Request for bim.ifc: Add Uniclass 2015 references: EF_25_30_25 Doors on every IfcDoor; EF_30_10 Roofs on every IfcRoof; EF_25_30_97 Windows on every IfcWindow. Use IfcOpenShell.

First a look at what the model holds.

```python
import ifcopenshell

model = ifcopenshell.open("bim.ifc")
print(model.schema)
print("classifications:", [c.Name for c in model.by_type("IfcClassification")])
for ifc_class in ("IfcDoor", "IfcRoof", "IfcStair", "IfcWall", "IfcWindow"):
    print(ifc_class, len(model.by_type(ifc_class)))
```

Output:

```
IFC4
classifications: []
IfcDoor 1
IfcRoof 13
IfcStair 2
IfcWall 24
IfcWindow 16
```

```python
import ifcopenshell
import ifcopenshell.api.classification

model = ifcopenshell.open("bim.ifc")

system = ifcopenshell.api.classification.add_classification(model, classification="Uniclass 2015")

codes = {
    "IfcDoor": ("EF_25_30_25", "Doors"),
    "IfcRoof": ("EF_30_10", "Roofs"),
    "IfcWindow": ("EF_25_30_97", "Windows"),
}
for ifc_class, (code, name) in codes.items():
    products = model.by_type(ifc_class)
    ifcopenshell.api.classification.add_reference(
        model, products=products, classification=system, identification=code, name=name
    )
    print(code, len(products))

model.write("bim-out.ifc")
```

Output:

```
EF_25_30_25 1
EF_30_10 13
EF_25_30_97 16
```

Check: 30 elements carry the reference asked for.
